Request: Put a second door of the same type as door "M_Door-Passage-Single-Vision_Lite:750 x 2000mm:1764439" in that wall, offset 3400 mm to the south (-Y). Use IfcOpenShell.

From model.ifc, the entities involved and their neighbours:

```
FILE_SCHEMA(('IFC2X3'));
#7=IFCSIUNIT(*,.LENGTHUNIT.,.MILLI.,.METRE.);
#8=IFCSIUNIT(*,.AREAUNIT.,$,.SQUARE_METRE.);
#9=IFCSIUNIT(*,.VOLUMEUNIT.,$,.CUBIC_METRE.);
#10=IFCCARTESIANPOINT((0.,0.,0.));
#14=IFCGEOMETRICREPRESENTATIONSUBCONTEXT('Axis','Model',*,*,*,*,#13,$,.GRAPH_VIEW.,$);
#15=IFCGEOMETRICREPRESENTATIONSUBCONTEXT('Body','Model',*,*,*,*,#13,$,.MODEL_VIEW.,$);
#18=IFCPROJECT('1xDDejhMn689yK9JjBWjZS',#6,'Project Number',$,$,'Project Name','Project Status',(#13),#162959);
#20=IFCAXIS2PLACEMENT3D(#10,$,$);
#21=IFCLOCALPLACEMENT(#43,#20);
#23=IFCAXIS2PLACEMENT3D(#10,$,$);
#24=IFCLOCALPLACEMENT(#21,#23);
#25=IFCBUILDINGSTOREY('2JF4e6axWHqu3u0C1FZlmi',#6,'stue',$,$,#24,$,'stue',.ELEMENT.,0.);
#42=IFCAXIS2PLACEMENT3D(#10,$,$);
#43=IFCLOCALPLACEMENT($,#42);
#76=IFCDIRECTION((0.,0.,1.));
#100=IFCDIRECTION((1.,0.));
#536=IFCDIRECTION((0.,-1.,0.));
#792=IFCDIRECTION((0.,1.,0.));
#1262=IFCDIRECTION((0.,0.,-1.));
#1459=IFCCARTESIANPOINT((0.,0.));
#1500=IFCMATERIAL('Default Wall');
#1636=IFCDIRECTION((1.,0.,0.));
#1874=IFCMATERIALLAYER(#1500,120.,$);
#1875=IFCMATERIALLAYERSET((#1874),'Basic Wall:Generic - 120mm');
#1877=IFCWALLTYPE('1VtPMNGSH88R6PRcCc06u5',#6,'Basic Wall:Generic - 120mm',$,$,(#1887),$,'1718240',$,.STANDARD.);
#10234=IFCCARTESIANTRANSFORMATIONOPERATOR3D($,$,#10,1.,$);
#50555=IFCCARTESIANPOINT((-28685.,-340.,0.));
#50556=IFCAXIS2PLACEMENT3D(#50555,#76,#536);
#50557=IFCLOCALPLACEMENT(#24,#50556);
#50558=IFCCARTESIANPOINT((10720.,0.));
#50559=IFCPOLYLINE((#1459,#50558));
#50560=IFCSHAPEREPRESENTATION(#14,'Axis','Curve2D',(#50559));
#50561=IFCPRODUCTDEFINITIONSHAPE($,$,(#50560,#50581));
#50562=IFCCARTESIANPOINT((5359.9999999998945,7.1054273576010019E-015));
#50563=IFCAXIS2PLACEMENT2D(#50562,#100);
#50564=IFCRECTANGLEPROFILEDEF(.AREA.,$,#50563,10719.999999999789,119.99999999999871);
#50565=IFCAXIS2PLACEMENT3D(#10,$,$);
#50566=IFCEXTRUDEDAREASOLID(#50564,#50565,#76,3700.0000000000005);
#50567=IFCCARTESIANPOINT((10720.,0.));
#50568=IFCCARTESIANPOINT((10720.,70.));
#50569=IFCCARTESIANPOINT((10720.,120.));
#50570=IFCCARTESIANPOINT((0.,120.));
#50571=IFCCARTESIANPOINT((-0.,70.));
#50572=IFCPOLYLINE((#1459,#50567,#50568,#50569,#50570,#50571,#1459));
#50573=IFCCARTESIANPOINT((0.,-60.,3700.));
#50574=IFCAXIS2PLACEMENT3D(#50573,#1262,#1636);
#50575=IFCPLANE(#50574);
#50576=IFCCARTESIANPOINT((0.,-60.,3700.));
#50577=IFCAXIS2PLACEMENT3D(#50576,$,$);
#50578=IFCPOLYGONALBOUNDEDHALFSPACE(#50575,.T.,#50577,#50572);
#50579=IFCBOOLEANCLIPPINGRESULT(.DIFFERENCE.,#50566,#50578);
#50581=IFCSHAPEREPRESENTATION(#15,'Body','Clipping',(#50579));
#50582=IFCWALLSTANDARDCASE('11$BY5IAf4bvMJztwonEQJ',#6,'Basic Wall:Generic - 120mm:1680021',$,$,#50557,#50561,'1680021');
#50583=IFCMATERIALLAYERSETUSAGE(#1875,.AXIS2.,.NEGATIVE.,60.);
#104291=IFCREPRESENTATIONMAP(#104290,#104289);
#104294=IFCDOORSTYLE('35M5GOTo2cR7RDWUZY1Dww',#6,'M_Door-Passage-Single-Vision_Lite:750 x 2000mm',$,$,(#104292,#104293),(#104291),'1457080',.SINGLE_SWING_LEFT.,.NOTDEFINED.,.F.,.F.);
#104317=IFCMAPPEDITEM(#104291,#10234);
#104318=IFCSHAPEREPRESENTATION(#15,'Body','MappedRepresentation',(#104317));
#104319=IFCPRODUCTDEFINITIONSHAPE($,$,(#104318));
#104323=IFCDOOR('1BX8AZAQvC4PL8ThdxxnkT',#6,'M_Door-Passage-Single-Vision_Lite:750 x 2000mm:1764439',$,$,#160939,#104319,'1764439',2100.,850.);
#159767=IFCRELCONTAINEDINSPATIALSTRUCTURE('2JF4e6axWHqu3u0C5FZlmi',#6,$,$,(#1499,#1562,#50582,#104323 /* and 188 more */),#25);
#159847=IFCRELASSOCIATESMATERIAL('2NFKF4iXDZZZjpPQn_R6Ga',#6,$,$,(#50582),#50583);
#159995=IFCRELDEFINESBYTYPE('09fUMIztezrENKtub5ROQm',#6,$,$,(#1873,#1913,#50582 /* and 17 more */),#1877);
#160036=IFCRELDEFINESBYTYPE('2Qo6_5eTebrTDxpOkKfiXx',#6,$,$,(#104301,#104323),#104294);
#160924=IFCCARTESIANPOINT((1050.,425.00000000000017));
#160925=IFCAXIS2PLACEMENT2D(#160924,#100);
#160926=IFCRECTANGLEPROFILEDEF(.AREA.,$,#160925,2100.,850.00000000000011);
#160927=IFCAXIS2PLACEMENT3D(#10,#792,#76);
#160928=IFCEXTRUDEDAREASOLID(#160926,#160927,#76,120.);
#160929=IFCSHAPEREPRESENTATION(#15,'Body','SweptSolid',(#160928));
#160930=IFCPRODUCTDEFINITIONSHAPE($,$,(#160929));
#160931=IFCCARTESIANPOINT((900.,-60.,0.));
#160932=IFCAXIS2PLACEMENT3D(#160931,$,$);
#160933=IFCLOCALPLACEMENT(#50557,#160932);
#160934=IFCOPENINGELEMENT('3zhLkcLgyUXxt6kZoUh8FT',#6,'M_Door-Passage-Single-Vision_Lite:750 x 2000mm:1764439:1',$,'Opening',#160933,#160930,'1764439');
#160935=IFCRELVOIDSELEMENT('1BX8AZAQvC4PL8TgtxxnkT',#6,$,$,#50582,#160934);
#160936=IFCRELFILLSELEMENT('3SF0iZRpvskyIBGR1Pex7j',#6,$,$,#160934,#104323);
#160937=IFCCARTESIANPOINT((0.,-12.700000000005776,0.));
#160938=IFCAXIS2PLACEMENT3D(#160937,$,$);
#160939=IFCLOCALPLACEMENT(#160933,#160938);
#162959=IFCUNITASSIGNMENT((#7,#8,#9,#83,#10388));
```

```python
import ifcopenshell
import ifcopenshell.api.feature
import ifcopenshell.api.geometry
import ifcopenshell.api.root
import ifcopenshell.geom
import ifcopenshell.util.element
import ifcopenshell.util.placement
import ifcopenshell.util.shape
import ifcopenshell.util.unit

model = ifcopenshell.open("model.ifc")
unit_scale = ifcopenshell.util.unit.calculate_unit_scale(model)
settings = ifcopenshell.geom.settings()


def volume(element):
    """Net volume in cubic metres, openings subtracted."""
    shape = ifcopenshell.geom.create_shape(settings, element)
    return ifcopenshell.util.shape.get_volume(shape.geometry)


def reuse_history(source, copy):
    """copy_class also copies each property set's owner history, people and application; keep the originals."""
    for rel in copy.IsDefinedBy:
        if rel.is_a("IfcRelDefinesByProperties") and (history := rel.RelatingPropertyDefinition.OwnerHistory):
            rel.RelatingPropertyDefinition.OwnerHistory = source.OwnerHistory
            ifcopenshell.util.element.remove_deep2(model, history)


door = model.by_guid("1BX8AZAQvC4PL8ThdxxnkT")
opening = door.FillsVoids[0].RelatingOpeningElement
wall = opening.VoidsElements[0].RelatingBuildingElement
before = volume(wall)
shift = ifcopenshell.util.placement.get_local_placement(wall.ObjectPlacement)[:3, 0] * 3.4 / unit_scale

# copy_class copies the void relationship, type, container and properties, but no geometry.
new_opening = ifcopenshell.api.root.copy_class(model, product=opening)
new_opening.Representation = ifcopenshell.util.element.copy_deep(
    model, opening.Representation, exclude=["IfcGeometricRepresentationContext", "IfcRepresentationMap"]
)
new_opening.Name = "M_Door-Passage-Single-Vision_Lite:750 x 2000mm"
new_opening.Tag = None
new_door = ifcopenshell.api.root.copy_class(model, product=door)
new_door.Representation = ifcopenshell.util.element.copy_deep(
    model, door.Representation, exclude=["IfcGeometricRepresentationContext", "IfcRepresentationMap"]
)
new_door.Name = "M_Door-Passage-Single-Vision_Lite:750 x 2000mm"
new_door.Tag = None
reuse_history(door, new_door)
fills = ifcopenshell.api.feature.add_filling(model, opening=new_opening, element=new_door)
fills.OwnerHistory = new_door.OwnerHistory  # required in IFC2X3

for old, new in ((opening, new_opening), (door, new_door)):
    matrix = ifcopenshell.util.placement.get_local_placement(old.ObjectPlacement)
    matrix[:3, 3] += shift
    ifcopenshell.api.geometry.edit_object_placement(model, product=new, matrix=matrix, is_si=False)

after = volume(wall)

print(f"wall volume {before:.3f} -> {after:.3f} m3")

model.write("model_v2.ifc")
```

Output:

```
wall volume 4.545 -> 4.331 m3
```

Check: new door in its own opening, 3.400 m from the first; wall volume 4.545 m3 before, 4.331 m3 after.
